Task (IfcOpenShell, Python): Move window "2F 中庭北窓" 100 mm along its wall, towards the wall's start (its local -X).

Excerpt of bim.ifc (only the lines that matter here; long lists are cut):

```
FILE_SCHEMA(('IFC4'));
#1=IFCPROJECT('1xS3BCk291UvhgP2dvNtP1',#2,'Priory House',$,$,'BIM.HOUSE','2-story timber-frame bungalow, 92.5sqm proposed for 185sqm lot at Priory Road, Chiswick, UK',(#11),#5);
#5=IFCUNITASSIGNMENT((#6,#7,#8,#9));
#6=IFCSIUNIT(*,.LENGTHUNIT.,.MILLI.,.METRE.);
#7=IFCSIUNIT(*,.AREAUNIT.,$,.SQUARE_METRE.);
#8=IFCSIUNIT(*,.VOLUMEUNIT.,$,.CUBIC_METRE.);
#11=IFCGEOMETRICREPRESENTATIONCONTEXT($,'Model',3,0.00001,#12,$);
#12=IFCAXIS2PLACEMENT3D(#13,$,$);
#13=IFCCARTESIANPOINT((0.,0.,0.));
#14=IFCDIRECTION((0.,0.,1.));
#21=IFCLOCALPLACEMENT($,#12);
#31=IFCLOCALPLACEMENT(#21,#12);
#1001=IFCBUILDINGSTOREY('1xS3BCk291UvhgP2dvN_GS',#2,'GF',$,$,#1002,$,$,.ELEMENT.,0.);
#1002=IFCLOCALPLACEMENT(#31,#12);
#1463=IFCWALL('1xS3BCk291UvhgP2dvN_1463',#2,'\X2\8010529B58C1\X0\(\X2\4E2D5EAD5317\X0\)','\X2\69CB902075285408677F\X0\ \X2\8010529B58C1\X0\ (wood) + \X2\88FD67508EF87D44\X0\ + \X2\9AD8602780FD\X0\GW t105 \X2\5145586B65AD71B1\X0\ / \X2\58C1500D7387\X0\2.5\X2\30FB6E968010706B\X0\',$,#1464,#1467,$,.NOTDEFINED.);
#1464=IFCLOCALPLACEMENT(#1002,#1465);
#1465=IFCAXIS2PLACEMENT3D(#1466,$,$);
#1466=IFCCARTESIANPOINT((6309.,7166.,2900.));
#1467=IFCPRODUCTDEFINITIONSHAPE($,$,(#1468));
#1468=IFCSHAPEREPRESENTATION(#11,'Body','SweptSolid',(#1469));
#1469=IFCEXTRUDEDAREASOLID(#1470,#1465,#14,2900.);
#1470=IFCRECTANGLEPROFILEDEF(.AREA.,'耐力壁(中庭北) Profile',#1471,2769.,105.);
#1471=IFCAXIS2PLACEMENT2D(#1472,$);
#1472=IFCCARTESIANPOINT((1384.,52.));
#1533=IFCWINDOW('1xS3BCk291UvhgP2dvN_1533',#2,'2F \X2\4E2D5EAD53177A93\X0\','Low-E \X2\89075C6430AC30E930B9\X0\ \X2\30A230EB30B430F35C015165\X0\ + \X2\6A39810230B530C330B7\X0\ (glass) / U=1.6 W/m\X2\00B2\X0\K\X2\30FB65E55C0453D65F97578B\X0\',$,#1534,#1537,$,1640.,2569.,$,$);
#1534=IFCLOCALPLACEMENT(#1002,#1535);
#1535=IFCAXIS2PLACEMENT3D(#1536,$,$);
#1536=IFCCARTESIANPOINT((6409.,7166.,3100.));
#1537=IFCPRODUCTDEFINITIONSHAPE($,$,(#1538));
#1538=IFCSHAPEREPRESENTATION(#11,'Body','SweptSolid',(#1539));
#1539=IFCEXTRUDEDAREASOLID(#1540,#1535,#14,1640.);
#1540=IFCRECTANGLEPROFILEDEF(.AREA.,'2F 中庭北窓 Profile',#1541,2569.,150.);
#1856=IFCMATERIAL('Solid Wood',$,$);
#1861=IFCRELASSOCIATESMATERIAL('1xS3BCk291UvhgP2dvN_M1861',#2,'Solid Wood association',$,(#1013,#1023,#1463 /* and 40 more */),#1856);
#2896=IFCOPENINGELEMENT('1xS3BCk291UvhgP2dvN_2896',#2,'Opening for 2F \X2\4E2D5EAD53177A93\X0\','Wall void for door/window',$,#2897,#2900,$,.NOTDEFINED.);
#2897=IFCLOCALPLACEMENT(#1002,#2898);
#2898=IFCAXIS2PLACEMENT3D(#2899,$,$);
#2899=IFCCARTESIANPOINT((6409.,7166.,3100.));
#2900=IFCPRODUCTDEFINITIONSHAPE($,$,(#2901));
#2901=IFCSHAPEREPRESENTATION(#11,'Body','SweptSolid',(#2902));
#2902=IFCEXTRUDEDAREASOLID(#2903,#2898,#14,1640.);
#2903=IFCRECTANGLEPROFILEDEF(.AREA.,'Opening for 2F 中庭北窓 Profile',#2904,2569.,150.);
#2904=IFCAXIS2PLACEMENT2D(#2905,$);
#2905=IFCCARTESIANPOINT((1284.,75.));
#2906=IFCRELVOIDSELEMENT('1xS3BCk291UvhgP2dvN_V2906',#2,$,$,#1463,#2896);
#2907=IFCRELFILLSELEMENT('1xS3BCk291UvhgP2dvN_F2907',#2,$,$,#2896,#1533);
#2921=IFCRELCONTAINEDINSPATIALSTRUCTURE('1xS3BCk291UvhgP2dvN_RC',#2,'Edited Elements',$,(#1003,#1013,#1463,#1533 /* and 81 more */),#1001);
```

```python
import ifcopenshell
import ifcopenshell.api.geometry
import ifcopenshell.util.placement
import ifcopenshell.util.unit

model = ifcopenshell.open("bim.ifc")
unit_scale = ifcopenshell.util.unit.calculate_unit_scale(model)

window = model.by_guid("1xS3BCk291UvhgP2dvN_1533")
opening = window.FillsVoids[0].RelatingOpeningElement
wall = opening.VoidsElements[0].RelatingBuildingElement

wall_matrix = ifcopenshell.util.placement.get_local_placement(wall.ObjectPlacement)
shift = wall_matrix[:3, 0] * -0.1 / unit_scale
before = ifcopenshell.util.placement.get_local_placement(window.ObjectPlacement)[:3, 3].copy()

# The window is not placed relative to its opening, so move both.
for product in (opening, window):
    matrix = ifcopenshell.util.placement.get_local_placement(product.ObjectPlacement)
    matrix[:3, 3] += shift
    ifcopenshell.api.geometry.edit_object_placement(model, product=product, matrix=matrix, is_si=False)

after = ifcopenshell.util.placement.get_local_placement(window.ObjectPlacement)[:3, 3]
print("window moved by", (after - before).round(3) + 0.0)

model.write("bim_v2.ifc")
```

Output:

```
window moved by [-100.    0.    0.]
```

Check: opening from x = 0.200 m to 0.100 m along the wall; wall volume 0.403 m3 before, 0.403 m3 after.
